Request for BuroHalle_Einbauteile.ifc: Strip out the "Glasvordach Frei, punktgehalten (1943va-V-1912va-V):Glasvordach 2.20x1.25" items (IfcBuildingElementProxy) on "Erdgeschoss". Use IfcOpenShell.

First a look at what the model holds.

```python
import ifcopenshell
import ifcopenshell.util.element

model = ifcopenshell.open("BuroHalle_Einbauteile.ifc")
print(model.schema)
storey = next(s for s in model.by_type("IfcBuildingStorey") if s.Name == "Erdgeschoss")
proxies = [e for e in ifcopenshell.util.element.get_decomposition(storey) if e.is_a("IfcBuildingElementProxy")]
seen = {}
for e in proxies:
    element_type = ifcopenshell.util.element.get_type(e)
    name = element_type.Name if element_type not in (None, e) else None
    seen[name] = seen.get(name, 0) + 1
for name, count in sorted(seen.items(), key=str):
    print(count, "x", name)
```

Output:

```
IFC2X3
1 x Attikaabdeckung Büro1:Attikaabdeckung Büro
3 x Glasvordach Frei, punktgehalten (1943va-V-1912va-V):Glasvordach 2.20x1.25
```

```python
import ifcopenshell
import ifcopenshell.api.root
import ifcopenshell.util.element

model = ifcopenshell.open("BuroHalle_Einbauteile.ifc")

storey = next(s for s in model.by_type("IfcBuildingStorey") if s.Name == "Erdgeschoss")
proxies = [e for e in ifcopenshell.util.element.get_decomposition(storey) if e.is_a("IfcBuildingElementProxy")]
targets = [e for e in proxies if (t := ifcopenshell.util.element.get_type(e)) not in (None, e) and t.Name == "Glasvordach Frei, punktgehalten (1943va-V-1912va-V):Glasvordach 2.20x1.25"]

for e in targets:
    ifcopenshell.api.root.remove_product(model, product=e)
print(len(targets), "removed")

model.write("BuroHalle_Einbauteile_v2.ifc")
```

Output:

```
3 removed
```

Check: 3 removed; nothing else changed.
